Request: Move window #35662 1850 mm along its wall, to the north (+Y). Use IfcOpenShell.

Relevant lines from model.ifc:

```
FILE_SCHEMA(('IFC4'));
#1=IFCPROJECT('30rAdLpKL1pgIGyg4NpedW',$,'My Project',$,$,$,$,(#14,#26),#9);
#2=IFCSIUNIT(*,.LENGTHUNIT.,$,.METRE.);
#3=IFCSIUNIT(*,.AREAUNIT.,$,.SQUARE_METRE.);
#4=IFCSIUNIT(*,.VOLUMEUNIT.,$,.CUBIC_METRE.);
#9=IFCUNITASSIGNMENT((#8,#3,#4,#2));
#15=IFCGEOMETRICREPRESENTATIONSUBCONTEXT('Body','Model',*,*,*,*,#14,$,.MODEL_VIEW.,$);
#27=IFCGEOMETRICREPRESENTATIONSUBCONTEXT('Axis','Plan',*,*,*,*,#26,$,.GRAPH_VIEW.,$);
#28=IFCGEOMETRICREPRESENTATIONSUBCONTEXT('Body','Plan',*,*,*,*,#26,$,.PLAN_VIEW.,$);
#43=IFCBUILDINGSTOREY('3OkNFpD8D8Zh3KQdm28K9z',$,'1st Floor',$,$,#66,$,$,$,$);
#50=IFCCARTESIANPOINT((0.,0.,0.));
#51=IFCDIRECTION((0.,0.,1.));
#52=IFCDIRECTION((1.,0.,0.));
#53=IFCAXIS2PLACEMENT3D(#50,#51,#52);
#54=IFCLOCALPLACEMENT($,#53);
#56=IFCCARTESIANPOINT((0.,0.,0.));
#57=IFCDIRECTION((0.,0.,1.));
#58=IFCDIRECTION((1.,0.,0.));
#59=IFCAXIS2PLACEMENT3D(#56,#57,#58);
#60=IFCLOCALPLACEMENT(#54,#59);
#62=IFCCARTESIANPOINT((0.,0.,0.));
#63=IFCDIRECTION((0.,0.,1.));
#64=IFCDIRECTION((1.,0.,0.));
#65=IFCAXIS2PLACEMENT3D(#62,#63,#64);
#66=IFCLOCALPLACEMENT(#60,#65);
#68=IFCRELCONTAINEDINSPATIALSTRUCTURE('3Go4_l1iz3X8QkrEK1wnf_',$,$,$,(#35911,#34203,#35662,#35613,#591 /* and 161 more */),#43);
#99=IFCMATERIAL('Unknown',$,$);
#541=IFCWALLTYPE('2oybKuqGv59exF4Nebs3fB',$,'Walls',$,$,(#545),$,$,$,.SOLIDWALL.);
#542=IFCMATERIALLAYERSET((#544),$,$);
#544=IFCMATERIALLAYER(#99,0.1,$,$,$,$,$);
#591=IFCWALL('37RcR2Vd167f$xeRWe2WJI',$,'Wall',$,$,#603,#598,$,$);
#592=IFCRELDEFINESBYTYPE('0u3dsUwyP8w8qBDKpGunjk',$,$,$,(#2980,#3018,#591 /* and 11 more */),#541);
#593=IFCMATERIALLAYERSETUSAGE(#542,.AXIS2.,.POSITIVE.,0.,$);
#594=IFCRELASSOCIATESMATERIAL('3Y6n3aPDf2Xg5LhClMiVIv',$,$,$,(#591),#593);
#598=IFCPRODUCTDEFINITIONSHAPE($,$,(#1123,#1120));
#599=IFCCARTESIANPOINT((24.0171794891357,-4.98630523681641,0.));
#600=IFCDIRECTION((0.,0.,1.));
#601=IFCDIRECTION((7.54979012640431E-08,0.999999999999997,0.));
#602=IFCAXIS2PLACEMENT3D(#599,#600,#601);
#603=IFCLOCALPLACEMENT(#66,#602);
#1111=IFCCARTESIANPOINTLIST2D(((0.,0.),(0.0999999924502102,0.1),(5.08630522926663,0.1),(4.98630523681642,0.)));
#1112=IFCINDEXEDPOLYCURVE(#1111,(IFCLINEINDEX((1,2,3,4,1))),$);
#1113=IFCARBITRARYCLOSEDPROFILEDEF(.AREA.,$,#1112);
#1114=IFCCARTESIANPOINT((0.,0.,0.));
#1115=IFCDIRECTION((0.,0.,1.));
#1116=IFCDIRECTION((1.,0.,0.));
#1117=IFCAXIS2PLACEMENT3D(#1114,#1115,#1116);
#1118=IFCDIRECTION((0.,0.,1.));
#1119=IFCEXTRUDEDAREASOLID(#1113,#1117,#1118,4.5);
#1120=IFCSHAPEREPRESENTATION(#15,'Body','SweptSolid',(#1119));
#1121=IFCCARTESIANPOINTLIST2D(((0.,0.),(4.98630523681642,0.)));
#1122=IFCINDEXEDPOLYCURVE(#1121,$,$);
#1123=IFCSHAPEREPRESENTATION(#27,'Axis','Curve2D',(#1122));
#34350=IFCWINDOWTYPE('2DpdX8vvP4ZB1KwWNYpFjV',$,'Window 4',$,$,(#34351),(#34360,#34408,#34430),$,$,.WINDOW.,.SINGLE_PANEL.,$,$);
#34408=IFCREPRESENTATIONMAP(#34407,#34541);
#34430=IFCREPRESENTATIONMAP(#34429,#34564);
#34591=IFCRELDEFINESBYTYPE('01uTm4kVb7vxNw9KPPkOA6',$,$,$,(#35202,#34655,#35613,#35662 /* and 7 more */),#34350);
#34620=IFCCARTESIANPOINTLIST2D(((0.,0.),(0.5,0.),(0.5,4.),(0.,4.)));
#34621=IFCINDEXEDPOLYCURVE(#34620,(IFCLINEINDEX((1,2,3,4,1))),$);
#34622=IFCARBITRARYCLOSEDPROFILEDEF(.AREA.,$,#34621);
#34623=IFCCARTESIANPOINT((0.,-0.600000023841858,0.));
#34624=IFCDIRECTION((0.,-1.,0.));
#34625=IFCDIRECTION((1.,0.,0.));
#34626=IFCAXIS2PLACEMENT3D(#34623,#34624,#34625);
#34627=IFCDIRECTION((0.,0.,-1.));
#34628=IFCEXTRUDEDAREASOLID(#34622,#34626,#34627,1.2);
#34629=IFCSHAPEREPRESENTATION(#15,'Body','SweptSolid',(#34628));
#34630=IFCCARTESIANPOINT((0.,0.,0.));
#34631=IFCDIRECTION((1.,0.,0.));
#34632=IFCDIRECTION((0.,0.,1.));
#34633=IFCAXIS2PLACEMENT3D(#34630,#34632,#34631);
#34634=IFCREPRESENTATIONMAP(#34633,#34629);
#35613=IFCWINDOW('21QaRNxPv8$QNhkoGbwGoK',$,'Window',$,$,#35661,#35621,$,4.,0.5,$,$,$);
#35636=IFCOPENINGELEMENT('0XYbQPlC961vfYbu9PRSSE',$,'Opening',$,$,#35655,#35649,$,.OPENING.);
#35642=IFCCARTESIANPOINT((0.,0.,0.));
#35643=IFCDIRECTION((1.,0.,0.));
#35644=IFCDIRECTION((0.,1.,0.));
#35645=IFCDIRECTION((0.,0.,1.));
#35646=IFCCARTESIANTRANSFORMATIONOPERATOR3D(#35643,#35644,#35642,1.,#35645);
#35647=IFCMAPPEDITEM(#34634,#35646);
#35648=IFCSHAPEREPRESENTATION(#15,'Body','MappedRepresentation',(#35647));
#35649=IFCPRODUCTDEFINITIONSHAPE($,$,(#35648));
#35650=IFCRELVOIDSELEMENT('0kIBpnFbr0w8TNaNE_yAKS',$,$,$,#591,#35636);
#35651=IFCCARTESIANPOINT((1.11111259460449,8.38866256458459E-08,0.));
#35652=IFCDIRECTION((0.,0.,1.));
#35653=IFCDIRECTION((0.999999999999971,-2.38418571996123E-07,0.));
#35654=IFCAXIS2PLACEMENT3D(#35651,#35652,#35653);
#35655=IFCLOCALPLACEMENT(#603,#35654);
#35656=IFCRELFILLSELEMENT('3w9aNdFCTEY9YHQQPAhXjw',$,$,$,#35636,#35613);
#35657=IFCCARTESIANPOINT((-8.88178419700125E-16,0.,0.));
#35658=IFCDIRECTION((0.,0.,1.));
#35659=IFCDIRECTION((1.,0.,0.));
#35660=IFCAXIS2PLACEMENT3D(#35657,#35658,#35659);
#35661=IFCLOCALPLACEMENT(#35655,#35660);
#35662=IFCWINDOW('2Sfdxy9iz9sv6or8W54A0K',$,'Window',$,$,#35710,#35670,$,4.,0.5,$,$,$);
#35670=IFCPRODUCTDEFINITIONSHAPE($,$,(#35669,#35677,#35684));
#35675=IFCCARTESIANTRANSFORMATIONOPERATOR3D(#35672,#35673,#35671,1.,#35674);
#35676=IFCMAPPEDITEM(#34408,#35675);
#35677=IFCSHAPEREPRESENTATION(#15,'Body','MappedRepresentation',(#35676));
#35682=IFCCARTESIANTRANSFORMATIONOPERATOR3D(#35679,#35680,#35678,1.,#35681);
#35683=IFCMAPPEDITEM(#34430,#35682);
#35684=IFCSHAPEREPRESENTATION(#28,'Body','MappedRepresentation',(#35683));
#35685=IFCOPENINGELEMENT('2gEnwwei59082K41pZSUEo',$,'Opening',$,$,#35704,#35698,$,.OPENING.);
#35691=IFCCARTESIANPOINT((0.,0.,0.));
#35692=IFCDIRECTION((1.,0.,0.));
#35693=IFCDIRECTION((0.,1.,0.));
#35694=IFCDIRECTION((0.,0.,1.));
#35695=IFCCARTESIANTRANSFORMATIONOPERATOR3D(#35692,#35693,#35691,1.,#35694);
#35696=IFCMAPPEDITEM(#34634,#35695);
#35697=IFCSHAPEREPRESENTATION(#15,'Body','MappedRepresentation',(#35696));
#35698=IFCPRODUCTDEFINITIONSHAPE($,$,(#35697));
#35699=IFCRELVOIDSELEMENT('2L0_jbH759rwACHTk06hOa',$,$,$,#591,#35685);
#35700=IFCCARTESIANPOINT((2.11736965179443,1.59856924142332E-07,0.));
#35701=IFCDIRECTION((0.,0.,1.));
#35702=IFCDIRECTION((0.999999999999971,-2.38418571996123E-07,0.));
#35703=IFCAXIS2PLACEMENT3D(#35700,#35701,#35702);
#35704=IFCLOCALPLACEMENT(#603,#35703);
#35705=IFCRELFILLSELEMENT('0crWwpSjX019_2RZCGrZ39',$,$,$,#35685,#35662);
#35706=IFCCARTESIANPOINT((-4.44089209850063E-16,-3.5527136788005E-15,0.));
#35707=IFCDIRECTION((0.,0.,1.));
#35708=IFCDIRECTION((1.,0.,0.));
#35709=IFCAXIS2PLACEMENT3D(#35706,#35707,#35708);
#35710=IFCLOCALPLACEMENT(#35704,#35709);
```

```python
import ifcopenshell
import ifcopenshell.api.geometry
import ifcopenshell.util.placement
import ifcopenshell.util.unit

model = ifcopenshell.open("model.ifc")
unit_scale = ifcopenshell.util.unit.calculate_unit_scale(model)

window = model.by_guid("2Sfdxy9iz9sv6or8W54A0K")
opening = window.FillsVoids[0].RelatingOpeningElement
wall = opening.VoidsElements[0].RelatingBuildingElement

wall_matrix = ifcopenshell.util.placement.get_local_placement(wall.ObjectPlacement)
shift = wall_matrix[:3, 0] * 1.85 / unit_scale
before = ifcopenshell.util.placement.get_local_placement(window.ObjectPlacement)[:3, 3].copy()

# The window is placed relative to its opening, so it follows when the opening moves.
matrix = ifcopenshell.util.placement.get_local_placement(opening.ObjectPlacement)
matrix[:3, 3] += shift
ifcopenshell.api.geometry.edit_object_placement(
    model, product=opening, matrix=matrix, is_si=False, should_transform_children=True
)

after = ifcopenshell.util.placement.get_local_placement(window.ObjectPlacement)[:3, 3]
print("window moved by", (after - before).round(3) + 0.0)

model.write("model_rev.ifc")
```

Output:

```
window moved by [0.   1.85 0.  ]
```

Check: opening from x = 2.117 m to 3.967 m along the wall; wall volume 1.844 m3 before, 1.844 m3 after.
